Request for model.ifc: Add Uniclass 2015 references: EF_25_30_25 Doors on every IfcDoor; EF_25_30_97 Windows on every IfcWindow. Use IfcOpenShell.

First a look at what the model holds.

```python
import ifcopenshell

model = ifcopenshell.open("model.ifc")
print(model.schema)
print("classifications:", [c.Name for c in model.by_type("IfcClassification")])
for ifc_class in ("IfcDoor", "IfcRoof", "IfcStair", "IfcWall", "IfcWindow"):
    print(ifc_class, len(model.by_type(ifc_class)))
```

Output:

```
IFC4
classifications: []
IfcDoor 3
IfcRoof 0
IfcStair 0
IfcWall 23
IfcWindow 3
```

```python
import ifcopenshell
import ifcopenshell.api.classification

model = ifcopenshell.open("model.ifc")

system = ifcopenshell.api.classification.add_classification(model, classification="Uniclass 2015")

codes = {
    "IfcDoor": ("EF_25_30_25", "Doors"),
    "IfcWindow": ("EF_25_30_97", "Windows"),
}
for ifc_class, (code, name) in codes.items():
    products = model.by_type(ifc_class)
    ifcopenshell.api.classification.add_reference(
        model, products=products, classification=system, identification=code, name=name
    )
    print(code, len(products))

model.write("model_edited.ifc")
```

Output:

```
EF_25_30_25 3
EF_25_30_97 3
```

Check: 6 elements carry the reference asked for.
